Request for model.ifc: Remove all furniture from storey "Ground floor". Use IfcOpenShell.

First a look at what the model holds.

```python
import ifcopenshell
import ifcopenshell.util.element

model = ifcopenshell.open("model.ifc")
print(model.schema)
storey = next(s for s in model.by_type("IfcBuildingStorey") if s.Name == "Ground floor")
furniture = [e for e in ifcopenshell.util.element.get_decomposition(storey) if e.is_a("IfcFurnishingElement")]
seen = {}
for e in furniture:
    element_type = ifcopenshell.util.element.get_type(e)
    name = element_type.Name if element_type not in (None, e) else None
    seen[name] = seen.get(name, 0) + 1
for name, count in sorted(seen.items(), key=str):
    print(count, "x", name)
```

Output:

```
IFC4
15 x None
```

```python
import ifcopenshell
import ifcopenshell.api.root
import ifcopenshell.util.element

model = ifcopenshell.open("model.ifc")

storey = next(s for s in model.by_type("IfcBuildingStorey") if s.Name == "Ground floor")
furniture = [e for e in ifcopenshell.util.element.get_decomposition(storey) if e.is_a("IfcFurnishingElement")]

for e in furniture:
    ifcopenshell.api.root.remove_product(model, product=e)
print(len(furniture), "removed")

model.write("model-out.ifc")
```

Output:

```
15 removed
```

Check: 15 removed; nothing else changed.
